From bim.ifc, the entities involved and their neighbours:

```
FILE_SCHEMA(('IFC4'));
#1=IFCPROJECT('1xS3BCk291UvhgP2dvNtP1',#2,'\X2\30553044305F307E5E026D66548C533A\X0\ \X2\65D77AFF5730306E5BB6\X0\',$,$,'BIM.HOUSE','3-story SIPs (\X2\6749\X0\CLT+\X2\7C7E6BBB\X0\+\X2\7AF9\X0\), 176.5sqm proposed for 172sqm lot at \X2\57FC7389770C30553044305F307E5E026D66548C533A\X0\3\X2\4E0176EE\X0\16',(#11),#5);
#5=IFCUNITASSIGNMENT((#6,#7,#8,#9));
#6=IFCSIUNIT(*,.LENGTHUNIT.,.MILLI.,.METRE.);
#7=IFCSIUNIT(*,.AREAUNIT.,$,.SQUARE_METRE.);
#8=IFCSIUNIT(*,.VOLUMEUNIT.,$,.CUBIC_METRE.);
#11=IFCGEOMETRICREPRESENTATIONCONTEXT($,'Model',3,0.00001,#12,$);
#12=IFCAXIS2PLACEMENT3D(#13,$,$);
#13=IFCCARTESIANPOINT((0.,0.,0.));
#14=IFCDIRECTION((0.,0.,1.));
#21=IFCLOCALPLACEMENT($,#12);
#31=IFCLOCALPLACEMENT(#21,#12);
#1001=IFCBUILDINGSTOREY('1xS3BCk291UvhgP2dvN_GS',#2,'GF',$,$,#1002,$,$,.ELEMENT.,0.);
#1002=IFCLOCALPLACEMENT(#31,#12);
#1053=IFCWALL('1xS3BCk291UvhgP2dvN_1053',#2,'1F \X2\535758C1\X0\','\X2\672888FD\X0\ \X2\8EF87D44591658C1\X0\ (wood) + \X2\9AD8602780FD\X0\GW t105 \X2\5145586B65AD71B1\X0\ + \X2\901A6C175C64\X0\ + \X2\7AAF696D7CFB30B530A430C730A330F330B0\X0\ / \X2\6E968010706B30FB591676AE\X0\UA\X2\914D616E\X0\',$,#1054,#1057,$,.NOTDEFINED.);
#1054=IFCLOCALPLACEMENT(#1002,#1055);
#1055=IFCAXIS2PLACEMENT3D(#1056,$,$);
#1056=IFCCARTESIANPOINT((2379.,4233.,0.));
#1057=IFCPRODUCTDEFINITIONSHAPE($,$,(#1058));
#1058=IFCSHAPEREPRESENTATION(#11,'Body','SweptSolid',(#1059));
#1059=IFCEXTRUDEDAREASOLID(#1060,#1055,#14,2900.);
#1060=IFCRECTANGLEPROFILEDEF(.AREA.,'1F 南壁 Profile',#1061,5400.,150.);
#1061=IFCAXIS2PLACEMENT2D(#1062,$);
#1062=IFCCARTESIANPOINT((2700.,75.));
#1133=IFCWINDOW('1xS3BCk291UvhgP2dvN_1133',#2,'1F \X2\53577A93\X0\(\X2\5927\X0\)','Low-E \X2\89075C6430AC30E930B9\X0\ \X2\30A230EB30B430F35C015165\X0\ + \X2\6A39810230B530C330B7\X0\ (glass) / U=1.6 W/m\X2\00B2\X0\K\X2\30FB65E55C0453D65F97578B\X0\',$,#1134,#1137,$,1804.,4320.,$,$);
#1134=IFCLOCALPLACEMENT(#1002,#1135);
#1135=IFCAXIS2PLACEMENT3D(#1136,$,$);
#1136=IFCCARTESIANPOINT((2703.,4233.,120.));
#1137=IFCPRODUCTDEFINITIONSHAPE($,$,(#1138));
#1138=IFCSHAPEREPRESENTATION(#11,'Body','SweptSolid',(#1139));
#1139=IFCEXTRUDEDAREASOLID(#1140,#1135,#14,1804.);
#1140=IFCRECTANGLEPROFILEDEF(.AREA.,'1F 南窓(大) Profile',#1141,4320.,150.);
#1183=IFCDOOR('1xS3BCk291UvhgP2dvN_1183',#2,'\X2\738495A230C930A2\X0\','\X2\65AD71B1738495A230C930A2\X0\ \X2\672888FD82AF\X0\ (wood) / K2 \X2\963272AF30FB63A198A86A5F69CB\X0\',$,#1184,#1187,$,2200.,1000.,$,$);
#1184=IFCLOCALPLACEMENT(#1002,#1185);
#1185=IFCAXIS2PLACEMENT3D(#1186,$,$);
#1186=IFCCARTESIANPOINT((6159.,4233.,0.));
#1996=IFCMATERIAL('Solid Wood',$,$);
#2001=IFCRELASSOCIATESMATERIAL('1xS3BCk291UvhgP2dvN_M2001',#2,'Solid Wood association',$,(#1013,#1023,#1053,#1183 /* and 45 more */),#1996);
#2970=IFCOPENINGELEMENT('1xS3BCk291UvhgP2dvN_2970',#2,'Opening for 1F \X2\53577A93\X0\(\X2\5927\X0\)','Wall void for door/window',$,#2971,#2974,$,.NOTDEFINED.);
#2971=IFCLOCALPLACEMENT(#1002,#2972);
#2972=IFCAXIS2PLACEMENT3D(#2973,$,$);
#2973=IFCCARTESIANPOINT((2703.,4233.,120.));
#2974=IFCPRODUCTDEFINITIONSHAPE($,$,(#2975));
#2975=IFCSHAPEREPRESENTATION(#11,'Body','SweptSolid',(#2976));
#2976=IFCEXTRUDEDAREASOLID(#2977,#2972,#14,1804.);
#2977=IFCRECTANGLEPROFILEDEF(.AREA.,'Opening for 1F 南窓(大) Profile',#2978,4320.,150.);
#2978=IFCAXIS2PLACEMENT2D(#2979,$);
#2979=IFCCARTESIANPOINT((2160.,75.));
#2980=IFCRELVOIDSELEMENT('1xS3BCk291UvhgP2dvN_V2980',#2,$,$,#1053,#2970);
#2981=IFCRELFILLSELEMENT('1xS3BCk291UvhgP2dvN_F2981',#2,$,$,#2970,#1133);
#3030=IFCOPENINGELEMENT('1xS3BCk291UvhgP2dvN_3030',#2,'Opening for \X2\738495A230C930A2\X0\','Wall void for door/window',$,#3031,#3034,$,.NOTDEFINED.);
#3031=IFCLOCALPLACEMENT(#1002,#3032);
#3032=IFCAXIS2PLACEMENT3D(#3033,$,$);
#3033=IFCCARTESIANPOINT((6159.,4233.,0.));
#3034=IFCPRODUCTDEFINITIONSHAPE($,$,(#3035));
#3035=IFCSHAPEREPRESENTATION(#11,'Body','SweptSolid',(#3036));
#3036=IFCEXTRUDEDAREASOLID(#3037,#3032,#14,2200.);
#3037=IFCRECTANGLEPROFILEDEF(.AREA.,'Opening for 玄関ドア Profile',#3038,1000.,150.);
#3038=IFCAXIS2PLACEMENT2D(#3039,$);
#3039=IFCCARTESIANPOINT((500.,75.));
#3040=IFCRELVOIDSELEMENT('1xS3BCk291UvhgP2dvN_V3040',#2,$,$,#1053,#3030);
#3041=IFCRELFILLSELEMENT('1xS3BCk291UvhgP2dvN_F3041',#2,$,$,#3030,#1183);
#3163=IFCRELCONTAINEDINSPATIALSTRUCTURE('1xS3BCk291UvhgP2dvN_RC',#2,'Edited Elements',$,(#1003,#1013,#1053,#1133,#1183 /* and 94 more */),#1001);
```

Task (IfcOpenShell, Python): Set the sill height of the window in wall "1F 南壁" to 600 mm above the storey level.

```python
import numpy as np
import ifcopenshell
import ifcopenshell.api.geometry
import ifcopenshell.geom
import ifcopenshell.util.element
import ifcopenshell.util.placement
import ifcopenshell.util.shape
import ifcopenshell.util.unit

model = ifcopenshell.open("bim.ifc")
unit_scale = ifcopenshell.util.unit.calculate_unit_scale(model)

window = model.by_id(1133)
opening = window.FillsVoids[0].RelatingOpeningElement
storey = ifcopenshell.util.element.get_container(window, ifc_class="IfcBuildingStorey")
level = ifcopenshell.util.placement.get_local_placement(storey.ObjectPlacement)[2, 3]

# The opening's origin need not be at the sill, so measure its lowest point.
shape = ifcopenshell.geom.create_shape(ifcopenshell.geom.settings(), opening)
bottom = ifcopenshell.util.shape.get_shape_bottom_elevation(shape, shape.geometry) / unit_scale
dz = level + 0.6 / unit_scale - bottom

shift = np.array([0.0, 0.0, dz])
# The window is not placed relative to its opening, so move both.
for product in (opening, window):
    matrix = ifcopenshell.util.placement.get_local_placement(product.ObjectPlacement)
    matrix[:3, 3] += shift
    ifcopenshell.api.geometry.edit_object_placement(model, product=product, matrix=matrix, is_si=False)

print(f"moved by {dz * unit_scale:+.3f} m")

model.write("bim_edited.ifc")
```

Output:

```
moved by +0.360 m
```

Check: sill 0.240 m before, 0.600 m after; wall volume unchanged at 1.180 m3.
